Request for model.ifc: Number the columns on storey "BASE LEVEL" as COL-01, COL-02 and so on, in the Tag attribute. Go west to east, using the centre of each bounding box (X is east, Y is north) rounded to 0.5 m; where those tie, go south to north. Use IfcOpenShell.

First a look at what the model holds.

```python
import ifcopenshell
import ifcopenshell.util.element
import ifcopenshell.util.placement

model = ifcopenshell.open("model.ifc")
print(model.schema)
storey = next(s for s in model.by_type("IfcBuildingStorey") if s.Name == "BASE LEVEL")
columns = [e for e in ifcopenshell.util.element.get_decomposition(storey) if e.is_a("IfcColumn")]
for e in sorted(columns, key=lambda e: e.id()):
    origin = ifcopenshell.util.placement.get_local_placement(e.ObjectPlacement)[:3, 3]
    print(e.id(), e.Tag, e.Name, origin.round(2) + 0.0, sep=" | ")
```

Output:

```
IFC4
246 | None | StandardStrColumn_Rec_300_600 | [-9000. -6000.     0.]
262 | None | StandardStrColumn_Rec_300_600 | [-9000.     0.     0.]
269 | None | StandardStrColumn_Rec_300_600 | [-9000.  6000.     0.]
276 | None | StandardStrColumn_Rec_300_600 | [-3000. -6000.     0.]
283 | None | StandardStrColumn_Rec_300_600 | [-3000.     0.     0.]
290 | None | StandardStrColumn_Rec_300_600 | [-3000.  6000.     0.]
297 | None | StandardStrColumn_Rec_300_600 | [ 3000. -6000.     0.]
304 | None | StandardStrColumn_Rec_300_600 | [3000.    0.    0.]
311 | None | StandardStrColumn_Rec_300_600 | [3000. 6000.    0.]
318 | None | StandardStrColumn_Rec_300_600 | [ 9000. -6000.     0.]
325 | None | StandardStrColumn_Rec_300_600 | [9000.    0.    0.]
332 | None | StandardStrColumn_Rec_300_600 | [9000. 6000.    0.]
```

```python
import ifcopenshell
import ifcopenshell.geom
import ifcopenshell.util.element
import ifcopenshell.util.shape

model = ifcopenshell.open("model.ifc")
settings = ifcopenshell.geom.settings()
settings.set("use-world-coords", True)


def centre(element):
    shape = ifcopenshell.geom.create_shape(settings, element)
    return ifcopenshell.util.shape.get_bbox_centroid(shape.geometry)


storey = next(s for s in model.by_type("IfcBuildingStorey") if s.Name == "BASE LEVEL")
columns = [e for e in ifcopenshell.util.element.get_decomposition(storey) if e.is_a("IfcColumn")]

# Insertion points can sit at a corner or the storey origin, so sort by the geometry (in metres).
centres = {e: centre(e) for e in columns}
columns.sort(key=lambda e: (round(centres[e][0] / 0.5), centres[e][1]))

for i, e in enumerate(columns, start=1):
    number = f"COL-{i:02d}"
    e.Tag = number
    print(e.id(), number)

model.write("model_updated.ifc")
```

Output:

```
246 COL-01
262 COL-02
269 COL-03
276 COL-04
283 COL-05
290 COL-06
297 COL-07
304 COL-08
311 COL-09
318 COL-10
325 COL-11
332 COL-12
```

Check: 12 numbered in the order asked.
